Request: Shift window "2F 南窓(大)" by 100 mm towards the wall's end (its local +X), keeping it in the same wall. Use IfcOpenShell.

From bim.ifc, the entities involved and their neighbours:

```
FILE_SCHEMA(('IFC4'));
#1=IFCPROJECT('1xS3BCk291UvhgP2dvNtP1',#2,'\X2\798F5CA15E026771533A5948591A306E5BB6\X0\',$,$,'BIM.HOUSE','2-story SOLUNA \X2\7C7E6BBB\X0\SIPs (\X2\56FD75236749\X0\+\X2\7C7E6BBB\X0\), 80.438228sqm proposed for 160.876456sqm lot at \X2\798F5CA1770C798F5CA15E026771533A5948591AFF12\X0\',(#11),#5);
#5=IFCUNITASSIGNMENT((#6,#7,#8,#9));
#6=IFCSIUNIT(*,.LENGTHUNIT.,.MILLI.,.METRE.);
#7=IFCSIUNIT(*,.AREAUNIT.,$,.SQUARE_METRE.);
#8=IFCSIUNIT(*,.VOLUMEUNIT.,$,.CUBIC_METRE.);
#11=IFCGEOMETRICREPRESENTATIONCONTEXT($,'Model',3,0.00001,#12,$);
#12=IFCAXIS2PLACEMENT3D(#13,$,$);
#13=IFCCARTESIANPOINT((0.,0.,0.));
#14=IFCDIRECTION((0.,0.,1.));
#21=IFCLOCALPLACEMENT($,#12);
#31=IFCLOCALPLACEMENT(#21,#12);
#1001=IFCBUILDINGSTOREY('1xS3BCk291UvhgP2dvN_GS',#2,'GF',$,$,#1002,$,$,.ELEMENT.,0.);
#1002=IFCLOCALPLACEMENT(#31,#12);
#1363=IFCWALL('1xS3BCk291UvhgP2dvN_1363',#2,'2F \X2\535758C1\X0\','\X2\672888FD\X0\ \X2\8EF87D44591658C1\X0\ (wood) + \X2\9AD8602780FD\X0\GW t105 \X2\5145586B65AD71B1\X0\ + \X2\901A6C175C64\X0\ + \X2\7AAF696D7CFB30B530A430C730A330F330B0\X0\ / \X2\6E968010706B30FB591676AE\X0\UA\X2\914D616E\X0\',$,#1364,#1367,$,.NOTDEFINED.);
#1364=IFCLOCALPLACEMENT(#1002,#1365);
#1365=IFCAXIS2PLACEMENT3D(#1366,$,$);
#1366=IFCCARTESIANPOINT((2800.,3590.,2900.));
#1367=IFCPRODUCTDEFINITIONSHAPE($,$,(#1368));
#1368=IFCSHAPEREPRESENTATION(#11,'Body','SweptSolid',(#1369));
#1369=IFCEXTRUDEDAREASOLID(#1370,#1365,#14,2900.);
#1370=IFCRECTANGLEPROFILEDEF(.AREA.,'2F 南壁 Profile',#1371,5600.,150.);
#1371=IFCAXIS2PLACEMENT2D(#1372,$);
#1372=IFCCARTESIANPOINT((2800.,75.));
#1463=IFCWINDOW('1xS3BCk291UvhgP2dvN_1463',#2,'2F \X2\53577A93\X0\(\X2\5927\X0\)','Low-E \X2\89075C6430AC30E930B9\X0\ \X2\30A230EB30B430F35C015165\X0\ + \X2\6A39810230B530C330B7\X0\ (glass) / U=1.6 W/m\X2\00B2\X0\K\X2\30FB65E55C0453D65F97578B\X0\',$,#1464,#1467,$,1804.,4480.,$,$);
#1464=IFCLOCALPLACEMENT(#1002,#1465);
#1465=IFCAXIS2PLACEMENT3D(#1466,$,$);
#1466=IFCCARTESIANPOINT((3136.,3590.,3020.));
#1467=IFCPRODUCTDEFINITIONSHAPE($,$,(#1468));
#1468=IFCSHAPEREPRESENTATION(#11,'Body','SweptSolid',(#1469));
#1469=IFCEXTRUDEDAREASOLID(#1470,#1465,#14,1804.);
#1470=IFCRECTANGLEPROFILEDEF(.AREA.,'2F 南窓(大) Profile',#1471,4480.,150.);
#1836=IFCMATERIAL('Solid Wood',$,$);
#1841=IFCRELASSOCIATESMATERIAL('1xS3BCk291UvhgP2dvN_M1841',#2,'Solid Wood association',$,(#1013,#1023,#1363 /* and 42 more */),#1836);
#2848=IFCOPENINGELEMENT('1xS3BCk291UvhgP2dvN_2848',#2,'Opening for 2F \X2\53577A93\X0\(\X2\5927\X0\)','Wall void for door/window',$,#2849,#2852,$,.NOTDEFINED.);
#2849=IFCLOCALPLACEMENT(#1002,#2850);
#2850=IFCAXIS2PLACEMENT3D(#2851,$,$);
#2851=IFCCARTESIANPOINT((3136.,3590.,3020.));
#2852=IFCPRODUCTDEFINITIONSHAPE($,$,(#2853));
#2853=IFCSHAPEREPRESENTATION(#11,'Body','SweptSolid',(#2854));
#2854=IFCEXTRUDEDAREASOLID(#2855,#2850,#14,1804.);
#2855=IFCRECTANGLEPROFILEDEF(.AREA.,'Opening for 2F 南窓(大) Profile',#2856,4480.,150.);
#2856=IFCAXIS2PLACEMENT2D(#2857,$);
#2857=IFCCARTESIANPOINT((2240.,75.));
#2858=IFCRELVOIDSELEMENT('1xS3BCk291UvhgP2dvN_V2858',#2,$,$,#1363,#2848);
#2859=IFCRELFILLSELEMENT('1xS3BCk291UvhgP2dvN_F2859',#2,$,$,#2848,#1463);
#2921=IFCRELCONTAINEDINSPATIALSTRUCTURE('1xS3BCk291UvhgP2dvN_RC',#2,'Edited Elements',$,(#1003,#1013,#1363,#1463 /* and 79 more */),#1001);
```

```python
import ifcopenshell
import ifcopenshell.api.geometry
import ifcopenshell.util.placement

model = ifcopenshell.open("bim.ifc")

window = model.by_guid("1xS3BCk291UvhgP2dvN_1463")
opening = window.FillsVoids[0].RelatingOpeningElement
wall = opening.VoidsElements[0].RelatingBuildingElement

wall_matrix = ifcopenshell.util.placement.get_local_placement(wall.ObjectPlacement)
shift = wall_matrix[:3, 0] * 100.0
before = ifcopenshell.util.placement.get_local_placement(window.ObjectPlacement)[:3, 3].copy()

# The window is not placed relative to its opening, so move both.
for product in (opening, window):
    matrix = ifcopenshell.util.placement.get_local_placement(product.ObjectPlacement)
    matrix[:3, 3] += shift
    ifcopenshell.api.geometry.edit_object_placement(model, product=product, matrix=matrix, is_si=False)

after = ifcopenshell.util.placement.get_local_placement(window.ObjectPlacement)[:3, 3]
print("window moved by", (after - before).round(3) + 0.0)

model.write("bim_updated.ifc")
```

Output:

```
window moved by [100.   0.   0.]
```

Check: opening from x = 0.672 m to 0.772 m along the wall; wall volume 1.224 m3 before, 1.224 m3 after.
